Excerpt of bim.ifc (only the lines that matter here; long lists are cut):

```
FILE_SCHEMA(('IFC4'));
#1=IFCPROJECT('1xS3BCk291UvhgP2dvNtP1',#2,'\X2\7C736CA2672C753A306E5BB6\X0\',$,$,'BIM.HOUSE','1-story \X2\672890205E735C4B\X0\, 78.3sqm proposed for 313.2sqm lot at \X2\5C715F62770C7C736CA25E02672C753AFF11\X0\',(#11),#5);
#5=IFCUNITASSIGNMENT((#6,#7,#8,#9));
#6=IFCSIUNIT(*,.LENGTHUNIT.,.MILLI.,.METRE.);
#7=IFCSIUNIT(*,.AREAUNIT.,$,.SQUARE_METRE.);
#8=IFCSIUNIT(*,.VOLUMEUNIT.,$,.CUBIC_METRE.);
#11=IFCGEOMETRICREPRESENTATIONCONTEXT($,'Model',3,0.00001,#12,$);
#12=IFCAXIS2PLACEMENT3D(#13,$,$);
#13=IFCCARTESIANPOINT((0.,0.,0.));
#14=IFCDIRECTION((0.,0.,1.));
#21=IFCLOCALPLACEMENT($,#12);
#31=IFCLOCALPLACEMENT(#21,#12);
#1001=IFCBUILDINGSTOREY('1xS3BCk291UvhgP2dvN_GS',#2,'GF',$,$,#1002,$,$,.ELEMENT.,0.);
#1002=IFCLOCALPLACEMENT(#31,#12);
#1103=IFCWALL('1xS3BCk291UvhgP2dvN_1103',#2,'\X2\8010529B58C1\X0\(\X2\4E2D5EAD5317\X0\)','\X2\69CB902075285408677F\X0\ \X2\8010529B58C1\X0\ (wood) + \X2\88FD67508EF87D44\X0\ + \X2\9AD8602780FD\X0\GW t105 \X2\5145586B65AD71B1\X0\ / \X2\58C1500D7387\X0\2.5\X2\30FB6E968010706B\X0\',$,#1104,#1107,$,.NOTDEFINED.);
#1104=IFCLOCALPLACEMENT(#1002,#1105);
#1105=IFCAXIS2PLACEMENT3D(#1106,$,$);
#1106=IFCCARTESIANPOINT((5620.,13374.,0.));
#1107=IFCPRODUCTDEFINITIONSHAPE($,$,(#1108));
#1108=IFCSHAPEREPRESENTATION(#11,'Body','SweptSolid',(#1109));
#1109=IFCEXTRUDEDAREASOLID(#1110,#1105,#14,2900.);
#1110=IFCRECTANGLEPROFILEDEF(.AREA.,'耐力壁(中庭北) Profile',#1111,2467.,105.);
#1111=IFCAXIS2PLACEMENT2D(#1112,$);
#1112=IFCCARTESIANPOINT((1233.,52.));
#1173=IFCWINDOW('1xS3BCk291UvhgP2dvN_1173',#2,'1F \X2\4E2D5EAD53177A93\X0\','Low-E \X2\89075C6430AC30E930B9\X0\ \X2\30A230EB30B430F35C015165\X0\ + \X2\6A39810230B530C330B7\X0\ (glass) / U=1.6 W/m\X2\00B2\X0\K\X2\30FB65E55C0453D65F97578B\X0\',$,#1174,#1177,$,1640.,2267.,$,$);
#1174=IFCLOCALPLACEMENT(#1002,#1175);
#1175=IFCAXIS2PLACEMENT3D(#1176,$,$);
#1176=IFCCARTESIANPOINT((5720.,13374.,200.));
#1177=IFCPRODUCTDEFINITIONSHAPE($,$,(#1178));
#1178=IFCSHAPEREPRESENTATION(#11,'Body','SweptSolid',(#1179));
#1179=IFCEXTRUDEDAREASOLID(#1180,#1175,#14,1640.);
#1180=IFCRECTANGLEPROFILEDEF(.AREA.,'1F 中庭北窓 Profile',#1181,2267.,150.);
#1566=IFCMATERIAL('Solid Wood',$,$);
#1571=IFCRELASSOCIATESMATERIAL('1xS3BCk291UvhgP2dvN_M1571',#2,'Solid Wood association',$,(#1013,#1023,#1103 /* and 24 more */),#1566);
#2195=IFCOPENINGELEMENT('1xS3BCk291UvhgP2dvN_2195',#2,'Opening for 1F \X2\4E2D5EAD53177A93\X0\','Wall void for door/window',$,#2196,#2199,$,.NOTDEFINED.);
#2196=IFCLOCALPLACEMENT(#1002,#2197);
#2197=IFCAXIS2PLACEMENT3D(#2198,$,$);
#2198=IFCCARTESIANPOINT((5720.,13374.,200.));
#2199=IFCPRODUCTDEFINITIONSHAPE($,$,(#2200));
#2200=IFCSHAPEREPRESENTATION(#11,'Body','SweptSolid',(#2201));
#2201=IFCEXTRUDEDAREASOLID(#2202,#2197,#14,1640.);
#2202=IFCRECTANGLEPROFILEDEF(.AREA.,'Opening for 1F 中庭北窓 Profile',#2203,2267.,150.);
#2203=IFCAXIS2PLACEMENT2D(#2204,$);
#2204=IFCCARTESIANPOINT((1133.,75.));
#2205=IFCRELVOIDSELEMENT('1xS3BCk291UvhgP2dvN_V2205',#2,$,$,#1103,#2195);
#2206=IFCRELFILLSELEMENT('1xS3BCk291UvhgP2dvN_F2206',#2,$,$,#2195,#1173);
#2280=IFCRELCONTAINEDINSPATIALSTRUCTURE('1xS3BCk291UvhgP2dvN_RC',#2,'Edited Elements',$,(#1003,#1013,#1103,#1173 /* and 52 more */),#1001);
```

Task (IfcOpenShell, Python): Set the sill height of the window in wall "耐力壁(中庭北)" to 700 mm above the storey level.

```python
import numpy as np
import ifcopenshell
import ifcopenshell.api.geometry
import ifcopenshell.geom
import ifcopenshell.util.element
import ifcopenshell.util.placement
import ifcopenshell.util.shape
import ifcopenshell.util.unit

model = ifcopenshell.open("bim.ifc")
unit_scale = ifcopenshell.util.unit.calculate_unit_scale(model)

window = model.by_guid("1xS3BCk291UvhgP2dvN_1173")
opening = window.FillsVoids[0].RelatingOpeningElement
storey = ifcopenshell.util.element.get_container(window, ifc_class="IfcBuildingStorey")
level = ifcopenshell.util.placement.get_local_placement(storey.ObjectPlacement)[2, 3]

# The opening's origin need not be at the sill, so measure its lowest point.
shape = ifcopenshell.geom.create_shape(ifcopenshell.geom.settings(), opening)
bottom = ifcopenshell.util.shape.get_shape_bottom_elevation(shape, shape.geometry) / unit_scale
dz = level + 0.7 / unit_scale - bottom

shift = np.array([0.0, 0.0, dz])
# The window is not placed relative to its opening, so move both.
for product in (opening, window):
    matrix = ifcopenshell.util.placement.get_local_placement(product.ObjectPlacement)
    matrix[:3, 3] += shift
    ifcopenshell.api.geometry.edit_object_placement(model, product=product, matrix=matrix, is_si=False)

print(f"moved by {dz * unit_scale:+.3f} m")

model.write("bim_updated.ifc")
```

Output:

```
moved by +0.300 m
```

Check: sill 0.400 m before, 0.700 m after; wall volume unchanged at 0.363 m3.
